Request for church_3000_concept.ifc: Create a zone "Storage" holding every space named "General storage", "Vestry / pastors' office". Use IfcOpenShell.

First a look at what the model holds.

```python
import ifcopenshell

model = ifcopenshell.open("church_3000_concept.ifc")
print(model.schema)
seen = {}
for space in model.by_type("IfcSpace"):
    seen[space.LongName] = seen.get(space.LongName, 0) + 1
for name, count in sorted(seen.items(), key=str):
    print(count, "x", name)
print("zones:", [z.Name for z in model.by_type("IfcZone")][:20])
```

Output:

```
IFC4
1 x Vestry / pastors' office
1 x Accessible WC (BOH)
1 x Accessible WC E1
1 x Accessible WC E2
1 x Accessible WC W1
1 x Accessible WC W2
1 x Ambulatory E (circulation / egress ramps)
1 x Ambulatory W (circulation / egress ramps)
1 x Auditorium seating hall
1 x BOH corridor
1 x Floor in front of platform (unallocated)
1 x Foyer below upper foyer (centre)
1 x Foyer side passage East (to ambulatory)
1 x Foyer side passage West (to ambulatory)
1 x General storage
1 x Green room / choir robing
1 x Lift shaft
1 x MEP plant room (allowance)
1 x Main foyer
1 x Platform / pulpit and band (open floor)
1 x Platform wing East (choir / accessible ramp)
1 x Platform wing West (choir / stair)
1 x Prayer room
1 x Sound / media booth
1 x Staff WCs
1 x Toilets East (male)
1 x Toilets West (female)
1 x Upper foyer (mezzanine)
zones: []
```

```python
import ifcopenshell
import ifcopenshell.api.group
import ifcopenshell.api.root

model = ifcopenshell.open("church_3000_concept.ifc")

names = {"General storage", "Vestry / pastors' office"}
spaces = [s for s in model.by_type("IfcSpace") if s.LongName in names]

zone = ifcopenshell.api.root.create_entity(model, ifc_class="IfcZone", name="Storage")
ifcopenshell.api.group.assign_group(model, products=spaces, group=zone)
print(len(spaces), "spaces in", zone.Name)

model.write("church_3000_concept_edited.ifc")
```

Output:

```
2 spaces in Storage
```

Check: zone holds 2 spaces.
